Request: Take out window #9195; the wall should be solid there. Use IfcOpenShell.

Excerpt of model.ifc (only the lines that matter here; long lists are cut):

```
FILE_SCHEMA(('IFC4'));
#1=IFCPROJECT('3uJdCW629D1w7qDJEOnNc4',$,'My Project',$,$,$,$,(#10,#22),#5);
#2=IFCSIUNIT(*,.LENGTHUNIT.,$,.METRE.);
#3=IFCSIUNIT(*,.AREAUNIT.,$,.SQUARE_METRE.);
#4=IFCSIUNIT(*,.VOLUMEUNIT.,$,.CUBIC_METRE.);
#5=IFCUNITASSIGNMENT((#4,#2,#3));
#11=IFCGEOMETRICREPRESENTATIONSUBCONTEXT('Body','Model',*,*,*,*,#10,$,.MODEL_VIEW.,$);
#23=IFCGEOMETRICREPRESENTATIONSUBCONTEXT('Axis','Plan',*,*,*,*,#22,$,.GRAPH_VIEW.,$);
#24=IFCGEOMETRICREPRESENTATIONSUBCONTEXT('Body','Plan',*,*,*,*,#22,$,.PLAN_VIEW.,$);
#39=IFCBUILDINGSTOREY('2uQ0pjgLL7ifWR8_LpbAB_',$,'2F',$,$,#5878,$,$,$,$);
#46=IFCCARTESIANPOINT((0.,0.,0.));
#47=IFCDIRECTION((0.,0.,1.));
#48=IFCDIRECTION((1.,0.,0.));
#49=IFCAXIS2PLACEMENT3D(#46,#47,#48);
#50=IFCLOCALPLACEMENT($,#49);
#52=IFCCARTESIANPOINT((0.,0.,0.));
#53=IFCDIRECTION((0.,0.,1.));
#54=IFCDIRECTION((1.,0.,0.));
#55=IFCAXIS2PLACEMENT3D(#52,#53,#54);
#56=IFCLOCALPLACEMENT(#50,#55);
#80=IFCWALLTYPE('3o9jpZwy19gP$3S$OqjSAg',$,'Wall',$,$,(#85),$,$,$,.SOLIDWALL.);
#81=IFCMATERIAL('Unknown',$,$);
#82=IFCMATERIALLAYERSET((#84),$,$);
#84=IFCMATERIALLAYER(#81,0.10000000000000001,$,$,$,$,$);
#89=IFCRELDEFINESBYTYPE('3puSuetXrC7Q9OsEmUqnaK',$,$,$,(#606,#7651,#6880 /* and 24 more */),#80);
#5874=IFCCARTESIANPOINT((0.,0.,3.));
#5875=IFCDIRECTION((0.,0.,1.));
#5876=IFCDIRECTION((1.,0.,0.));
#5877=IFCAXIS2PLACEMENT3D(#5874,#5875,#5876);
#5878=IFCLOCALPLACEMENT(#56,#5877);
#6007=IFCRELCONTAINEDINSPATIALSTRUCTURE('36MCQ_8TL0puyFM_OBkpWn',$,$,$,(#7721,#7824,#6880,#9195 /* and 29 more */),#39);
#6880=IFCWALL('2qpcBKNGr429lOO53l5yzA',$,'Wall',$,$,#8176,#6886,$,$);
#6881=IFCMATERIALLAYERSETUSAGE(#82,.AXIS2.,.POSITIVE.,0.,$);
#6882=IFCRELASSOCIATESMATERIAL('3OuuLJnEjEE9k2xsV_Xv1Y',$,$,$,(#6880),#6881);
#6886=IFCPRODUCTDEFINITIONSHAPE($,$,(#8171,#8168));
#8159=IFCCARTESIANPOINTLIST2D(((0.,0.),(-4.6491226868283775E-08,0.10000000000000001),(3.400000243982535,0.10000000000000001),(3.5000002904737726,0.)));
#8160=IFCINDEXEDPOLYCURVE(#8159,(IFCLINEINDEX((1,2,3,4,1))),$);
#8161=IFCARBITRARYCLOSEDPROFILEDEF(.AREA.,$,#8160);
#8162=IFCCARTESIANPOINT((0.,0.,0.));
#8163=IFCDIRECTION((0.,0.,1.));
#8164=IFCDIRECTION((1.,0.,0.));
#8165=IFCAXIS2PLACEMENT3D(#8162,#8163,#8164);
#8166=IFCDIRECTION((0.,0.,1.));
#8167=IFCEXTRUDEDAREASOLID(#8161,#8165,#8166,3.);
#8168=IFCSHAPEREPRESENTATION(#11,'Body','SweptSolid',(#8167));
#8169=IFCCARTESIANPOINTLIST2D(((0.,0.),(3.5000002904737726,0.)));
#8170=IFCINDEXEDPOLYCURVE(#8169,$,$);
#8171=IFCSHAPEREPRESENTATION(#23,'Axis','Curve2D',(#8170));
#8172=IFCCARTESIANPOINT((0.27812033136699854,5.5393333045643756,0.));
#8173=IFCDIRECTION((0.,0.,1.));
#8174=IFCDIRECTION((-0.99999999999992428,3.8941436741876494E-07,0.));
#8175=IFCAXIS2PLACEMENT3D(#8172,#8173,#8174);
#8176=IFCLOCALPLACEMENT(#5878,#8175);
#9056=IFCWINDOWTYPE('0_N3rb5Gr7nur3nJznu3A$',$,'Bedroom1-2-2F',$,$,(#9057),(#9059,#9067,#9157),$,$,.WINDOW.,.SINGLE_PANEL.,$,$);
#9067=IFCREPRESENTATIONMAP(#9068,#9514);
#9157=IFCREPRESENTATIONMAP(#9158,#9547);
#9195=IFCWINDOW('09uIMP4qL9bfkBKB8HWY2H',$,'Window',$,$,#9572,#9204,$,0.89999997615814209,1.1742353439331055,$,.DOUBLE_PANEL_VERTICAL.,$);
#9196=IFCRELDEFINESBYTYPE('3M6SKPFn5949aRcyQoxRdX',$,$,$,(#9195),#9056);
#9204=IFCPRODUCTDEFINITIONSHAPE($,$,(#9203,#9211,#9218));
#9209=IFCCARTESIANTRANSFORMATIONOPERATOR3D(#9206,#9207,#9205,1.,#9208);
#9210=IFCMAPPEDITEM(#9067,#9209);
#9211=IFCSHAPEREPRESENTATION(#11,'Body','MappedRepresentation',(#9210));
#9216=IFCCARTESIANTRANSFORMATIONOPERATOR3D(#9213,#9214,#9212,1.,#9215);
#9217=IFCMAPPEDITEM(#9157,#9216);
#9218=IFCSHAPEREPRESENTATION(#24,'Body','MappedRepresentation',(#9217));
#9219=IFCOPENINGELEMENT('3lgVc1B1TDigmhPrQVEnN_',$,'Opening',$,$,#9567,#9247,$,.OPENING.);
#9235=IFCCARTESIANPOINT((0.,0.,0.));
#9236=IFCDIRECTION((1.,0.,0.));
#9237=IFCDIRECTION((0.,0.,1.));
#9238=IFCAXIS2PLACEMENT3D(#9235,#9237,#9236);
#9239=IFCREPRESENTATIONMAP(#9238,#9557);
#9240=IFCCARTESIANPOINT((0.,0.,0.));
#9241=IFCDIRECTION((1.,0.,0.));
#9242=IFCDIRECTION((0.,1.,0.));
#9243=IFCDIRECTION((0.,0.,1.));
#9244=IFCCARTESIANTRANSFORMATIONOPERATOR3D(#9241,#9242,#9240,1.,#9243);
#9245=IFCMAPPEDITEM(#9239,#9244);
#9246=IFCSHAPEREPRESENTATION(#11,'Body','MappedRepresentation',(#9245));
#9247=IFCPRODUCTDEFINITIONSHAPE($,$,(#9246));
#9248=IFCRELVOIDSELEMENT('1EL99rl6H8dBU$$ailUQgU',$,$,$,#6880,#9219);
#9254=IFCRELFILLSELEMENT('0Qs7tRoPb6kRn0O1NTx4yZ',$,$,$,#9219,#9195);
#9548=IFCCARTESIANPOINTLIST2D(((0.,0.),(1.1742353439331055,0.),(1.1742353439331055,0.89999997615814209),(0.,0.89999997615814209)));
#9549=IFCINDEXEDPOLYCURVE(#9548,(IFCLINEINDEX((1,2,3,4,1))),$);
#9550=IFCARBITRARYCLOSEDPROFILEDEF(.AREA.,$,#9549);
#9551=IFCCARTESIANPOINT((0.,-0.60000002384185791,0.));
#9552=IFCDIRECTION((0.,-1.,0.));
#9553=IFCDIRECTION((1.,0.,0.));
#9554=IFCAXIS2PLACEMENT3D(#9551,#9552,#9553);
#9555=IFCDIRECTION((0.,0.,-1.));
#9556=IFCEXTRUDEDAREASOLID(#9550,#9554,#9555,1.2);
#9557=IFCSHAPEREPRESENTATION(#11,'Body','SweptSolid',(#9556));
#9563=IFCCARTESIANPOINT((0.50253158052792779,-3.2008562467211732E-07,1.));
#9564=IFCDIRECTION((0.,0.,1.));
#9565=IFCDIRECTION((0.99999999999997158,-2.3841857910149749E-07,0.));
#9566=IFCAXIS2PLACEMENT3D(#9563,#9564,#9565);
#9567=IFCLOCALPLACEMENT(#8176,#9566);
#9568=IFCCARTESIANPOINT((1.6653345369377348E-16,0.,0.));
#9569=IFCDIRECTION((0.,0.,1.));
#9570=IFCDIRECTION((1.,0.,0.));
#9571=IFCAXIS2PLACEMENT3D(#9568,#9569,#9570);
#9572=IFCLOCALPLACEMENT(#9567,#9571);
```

```python
import ifcopenshell
import ifcopenshell.api.feature
import ifcopenshell.api.root
import ifcopenshell.geom
import ifcopenshell.util.shape

model = ifcopenshell.open("model.ifc")
settings = ifcopenshell.geom.settings()


def volume(element):
    """Net volume in cubic metres, openings subtracted."""
    shape = ifcopenshell.geom.create_shape(settings, element)
    return ifcopenshell.util.shape.get_volume(shape.geometry)


window = model.by_guid("09uIMP4qL9bfkBKB8HWY2H")
opening = window.FillsVoids[0].RelatingOpeningElement
wall = opening.VoidsElements[0].RelatingBuildingElement
before = volume(wall)

ifcopenshell.api.root.remove_product(model, product=window)
ifcopenshell.api.feature.remove_feature(model, feature=opening)

after = volume(wall)

print(f"wall volume {before:.3f} -> {after:.3f} m3")

model.write("model_v2.ifc")
```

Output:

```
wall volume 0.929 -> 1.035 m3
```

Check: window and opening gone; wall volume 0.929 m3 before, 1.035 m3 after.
